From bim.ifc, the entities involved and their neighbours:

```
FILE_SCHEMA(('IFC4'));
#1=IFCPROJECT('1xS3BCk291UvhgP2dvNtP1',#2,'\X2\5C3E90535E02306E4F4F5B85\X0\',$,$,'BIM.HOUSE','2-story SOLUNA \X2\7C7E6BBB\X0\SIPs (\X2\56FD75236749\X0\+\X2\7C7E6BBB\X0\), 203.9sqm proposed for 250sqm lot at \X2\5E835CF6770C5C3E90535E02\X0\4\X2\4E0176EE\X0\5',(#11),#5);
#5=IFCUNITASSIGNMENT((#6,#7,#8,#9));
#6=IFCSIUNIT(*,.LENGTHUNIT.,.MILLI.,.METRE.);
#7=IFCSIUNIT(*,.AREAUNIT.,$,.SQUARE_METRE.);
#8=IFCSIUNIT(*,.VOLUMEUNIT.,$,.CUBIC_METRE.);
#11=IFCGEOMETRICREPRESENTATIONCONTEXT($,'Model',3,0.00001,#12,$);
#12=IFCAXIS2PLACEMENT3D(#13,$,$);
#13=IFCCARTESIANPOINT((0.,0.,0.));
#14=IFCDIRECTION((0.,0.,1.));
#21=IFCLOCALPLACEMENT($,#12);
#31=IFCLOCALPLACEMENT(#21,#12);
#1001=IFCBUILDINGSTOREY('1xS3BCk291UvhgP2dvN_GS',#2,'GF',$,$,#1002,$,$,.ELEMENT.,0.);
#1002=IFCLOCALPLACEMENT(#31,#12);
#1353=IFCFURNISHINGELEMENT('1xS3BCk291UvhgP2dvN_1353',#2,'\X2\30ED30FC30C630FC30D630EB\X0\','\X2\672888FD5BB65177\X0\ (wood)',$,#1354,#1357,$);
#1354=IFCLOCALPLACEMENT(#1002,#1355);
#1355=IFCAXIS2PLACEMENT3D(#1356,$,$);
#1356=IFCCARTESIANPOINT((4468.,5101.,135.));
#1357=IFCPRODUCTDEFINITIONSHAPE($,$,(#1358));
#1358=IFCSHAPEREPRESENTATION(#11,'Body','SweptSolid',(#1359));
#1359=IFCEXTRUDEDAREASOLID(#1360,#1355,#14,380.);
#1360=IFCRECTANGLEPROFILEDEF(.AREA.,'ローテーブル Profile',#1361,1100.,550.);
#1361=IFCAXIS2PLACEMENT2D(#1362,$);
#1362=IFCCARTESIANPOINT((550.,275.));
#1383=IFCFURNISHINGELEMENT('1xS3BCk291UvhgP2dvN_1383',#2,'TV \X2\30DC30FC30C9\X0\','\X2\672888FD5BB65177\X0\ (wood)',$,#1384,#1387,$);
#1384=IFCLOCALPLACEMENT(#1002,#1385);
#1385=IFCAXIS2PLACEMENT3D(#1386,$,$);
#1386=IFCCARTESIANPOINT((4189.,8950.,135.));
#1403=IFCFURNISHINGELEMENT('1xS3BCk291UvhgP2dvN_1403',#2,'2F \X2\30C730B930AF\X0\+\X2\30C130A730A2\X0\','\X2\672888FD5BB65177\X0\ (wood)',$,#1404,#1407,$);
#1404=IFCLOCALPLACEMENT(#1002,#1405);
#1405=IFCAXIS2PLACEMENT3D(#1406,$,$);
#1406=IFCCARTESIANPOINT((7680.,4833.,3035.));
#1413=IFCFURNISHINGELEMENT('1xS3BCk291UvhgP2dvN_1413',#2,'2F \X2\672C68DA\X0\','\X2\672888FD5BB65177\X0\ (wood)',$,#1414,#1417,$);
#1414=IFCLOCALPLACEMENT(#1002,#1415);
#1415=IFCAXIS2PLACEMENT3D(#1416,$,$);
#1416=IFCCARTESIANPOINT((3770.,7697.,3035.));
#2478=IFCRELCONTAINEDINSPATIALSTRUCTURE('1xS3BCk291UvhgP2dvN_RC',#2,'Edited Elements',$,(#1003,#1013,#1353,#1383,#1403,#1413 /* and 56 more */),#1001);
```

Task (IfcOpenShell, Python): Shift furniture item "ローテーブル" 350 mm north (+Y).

```python
import ifcopenshell
import ifcopenshell.api.geometry
import ifcopenshell.util.placement
import ifcopenshell.util.unit

model = ifcopenshell.open("bim.ifc")
unit_scale = ifcopenshell.util.unit.calculate_unit_scale(model)

item = model.by_id(1353)
matrix = ifcopenshell.util.placement.get_local_placement(item.ObjectPlacement)
matrix[1, 3] += 0.35 / unit_scale
ifcopenshell.api.geometry.edit_object_placement(model, product=item, matrix=matrix, is_si=False)

print(ifcopenshell.util.placement.get_local_placement(item.ObjectPlacement).round(3) + 0.0)

model.write("bim_v2.ifc")
```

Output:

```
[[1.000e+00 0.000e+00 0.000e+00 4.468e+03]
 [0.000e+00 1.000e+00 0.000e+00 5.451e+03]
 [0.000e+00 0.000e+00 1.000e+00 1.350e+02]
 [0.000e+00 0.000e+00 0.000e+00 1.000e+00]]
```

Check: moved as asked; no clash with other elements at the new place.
